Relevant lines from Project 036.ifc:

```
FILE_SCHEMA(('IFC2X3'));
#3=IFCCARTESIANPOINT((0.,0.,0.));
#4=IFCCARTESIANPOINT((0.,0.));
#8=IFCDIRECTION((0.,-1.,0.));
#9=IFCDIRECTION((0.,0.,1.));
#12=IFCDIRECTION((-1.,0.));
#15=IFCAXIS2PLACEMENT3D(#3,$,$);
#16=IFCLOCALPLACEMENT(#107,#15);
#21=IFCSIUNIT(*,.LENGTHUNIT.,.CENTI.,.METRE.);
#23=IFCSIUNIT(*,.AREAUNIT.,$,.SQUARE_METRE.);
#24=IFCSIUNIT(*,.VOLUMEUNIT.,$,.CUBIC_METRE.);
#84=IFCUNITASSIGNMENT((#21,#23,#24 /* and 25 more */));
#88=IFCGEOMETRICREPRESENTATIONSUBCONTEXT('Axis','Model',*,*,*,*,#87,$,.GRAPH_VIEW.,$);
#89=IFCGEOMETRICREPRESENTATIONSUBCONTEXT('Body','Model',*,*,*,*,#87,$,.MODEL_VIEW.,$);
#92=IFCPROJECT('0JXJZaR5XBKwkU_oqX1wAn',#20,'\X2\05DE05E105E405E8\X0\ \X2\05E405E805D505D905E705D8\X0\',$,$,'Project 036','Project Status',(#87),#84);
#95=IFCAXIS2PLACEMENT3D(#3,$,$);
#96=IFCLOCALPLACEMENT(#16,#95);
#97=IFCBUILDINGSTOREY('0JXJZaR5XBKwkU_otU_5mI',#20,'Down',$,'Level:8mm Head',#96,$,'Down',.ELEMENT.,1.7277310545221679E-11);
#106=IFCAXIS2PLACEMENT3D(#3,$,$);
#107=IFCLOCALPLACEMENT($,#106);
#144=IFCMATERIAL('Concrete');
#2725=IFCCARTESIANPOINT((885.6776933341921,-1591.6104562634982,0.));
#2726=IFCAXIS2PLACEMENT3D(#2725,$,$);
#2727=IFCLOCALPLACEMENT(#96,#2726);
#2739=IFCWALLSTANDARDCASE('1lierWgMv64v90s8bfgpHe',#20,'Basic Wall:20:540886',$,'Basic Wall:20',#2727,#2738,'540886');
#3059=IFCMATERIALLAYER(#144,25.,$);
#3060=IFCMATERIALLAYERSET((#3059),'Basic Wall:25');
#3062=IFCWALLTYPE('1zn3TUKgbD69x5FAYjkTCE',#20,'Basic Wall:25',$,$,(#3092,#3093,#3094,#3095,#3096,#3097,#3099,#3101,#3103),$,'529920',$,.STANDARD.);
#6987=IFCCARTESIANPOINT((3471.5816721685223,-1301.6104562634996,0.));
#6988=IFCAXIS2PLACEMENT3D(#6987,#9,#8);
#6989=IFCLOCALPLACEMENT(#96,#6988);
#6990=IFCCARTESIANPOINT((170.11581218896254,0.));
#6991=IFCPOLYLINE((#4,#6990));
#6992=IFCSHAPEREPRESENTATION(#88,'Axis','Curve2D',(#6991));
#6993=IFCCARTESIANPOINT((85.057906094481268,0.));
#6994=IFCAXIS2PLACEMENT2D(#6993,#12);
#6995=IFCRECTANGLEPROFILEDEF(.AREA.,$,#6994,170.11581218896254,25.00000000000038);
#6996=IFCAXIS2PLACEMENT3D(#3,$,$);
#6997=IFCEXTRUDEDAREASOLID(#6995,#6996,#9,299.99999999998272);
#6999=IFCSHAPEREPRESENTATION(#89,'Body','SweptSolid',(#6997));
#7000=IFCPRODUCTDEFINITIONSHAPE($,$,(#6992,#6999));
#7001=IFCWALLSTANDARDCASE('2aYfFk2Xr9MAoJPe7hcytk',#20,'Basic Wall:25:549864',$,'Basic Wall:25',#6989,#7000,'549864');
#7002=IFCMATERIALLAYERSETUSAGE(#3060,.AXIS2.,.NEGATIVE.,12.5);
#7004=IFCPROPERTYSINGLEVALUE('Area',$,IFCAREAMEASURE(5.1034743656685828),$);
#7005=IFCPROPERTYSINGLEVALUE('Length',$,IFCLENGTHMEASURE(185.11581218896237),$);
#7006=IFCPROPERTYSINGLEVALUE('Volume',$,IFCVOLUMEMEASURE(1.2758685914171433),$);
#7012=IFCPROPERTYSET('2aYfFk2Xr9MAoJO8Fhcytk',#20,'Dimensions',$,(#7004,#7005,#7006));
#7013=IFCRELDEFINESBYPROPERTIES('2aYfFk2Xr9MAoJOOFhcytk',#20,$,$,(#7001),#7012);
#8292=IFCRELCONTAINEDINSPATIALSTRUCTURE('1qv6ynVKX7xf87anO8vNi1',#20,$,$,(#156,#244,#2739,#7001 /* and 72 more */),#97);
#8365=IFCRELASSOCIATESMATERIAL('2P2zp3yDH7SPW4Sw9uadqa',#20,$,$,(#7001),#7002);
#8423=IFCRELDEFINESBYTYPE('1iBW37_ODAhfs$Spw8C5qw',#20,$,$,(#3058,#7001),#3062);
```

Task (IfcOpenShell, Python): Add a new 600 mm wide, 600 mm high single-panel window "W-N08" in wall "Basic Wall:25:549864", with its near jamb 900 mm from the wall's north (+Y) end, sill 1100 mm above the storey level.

```python
import numpy as np
import ifcopenshell
import ifcopenshell.api.feature
import ifcopenshell.api.geometry
import ifcopenshell.api.pset
import ifcopenshell.api.root
import ifcopenshell.api.spatial
import ifcopenshell.api.type
import ifcopenshell.geom
import ifcopenshell.util.element
import ifcopenshell.util.placement
import ifcopenshell.util.representation
import ifcopenshell.util.shape
import ifcopenshell.util.unit

model = ifcopenshell.open("Project 036.ifc")
unit_scale = ifcopenshell.util.unit.calculate_unit_scale(model)
area_scale = ifcopenshell.util.unit.calculate_unit_scale(model, "AREAUNIT")
volume_scale = ifcopenshell.util.unit.calculate_unit_scale(model, "VOLUMEUNIT")
settings = ifcopenshell.geom.settings()


def volume(element):
    """Net volume in cubic metres, openings subtracted."""
    shape = ifcopenshell.geom.create_shape(settings, element)
    return ifcopenshell.util.shape.get_volume(shape.geometry)


wall = model.by_guid("2aYfFk2Xr9MAoJPe7hcytk")
storey = ifcopenshell.util.element.get_container(wall, ifc_class="IfcBuildingStorey")
context = ifcopenshell.util.representation.get_context(model, "Model", "Body", "MODEL_VIEW")
before = volume(wall)

width, height, from_end, sill = 0.6, 0.6, 0.9, 1.1  # metres

# The wall runs along its own X axis, and the end named is its -X end.
wall_shape = ifcopenshell.geom.create_shape(settings, wall)
x, y, z = ifcopenshell.util.shape.get_vertices(wall_shape.geometry).T
start = x.min() + from_end
face, thickness = float(y.min()), float(y.max() - y.min())
wall_matrix = ifcopenshell.util.placement.get_local_placement(wall.ObjectPlacement)
level = ifcopenshell.util.placement.get_local_placement(storey.ObjectPlacement)[2, 3]


def in_wall(x, y):
    """Placement at x, y metres in the wall's axes, at sill height."""
    matrix = wall_matrix.copy()
    matrix[:, 3] = wall_matrix @ np.array([x / unit_scale, y / unit_scale, 0.0, 1.0])
    matrix[2, 3] = level + sill / unit_scale
    return matrix


# Opening: a box that overshoots both wall faces by 50 mm.
opening = ifcopenshell.api.root.create_entity(model, ifc_class="IfcOpeningElement")
box = ifcopenshell.api.geometry.add_wall_representation(
    model, context=context, length=width, height=height, thickness=thickness + 0.1
)
ifcopenshell.api.geometry.assign_representation(model, product=opening, representation=box)
ifcopenshell.api.geometry.edit_object_placement(model, product=opening, matrix=in_wall(start, face - 0.05), is_si=False)
ifcopenshell.api.feature.add_feature(model, feature=opening, element=wall)

window = ifcopenshell.api.root.create_entity(model, ifc_class="IfcWindow", name="W-N08")
window.OverallWidth, window.OverallHeight = width / unit_scale, height / unit_scale
body = ifcopenshell.api.geometry.add_window_representation(
    model,
    context=context,
    overall_width=window.OverallWidth,
    overall_height=window.OverallHeight,
    partition_type="SINGLE_PANEL",
)
ifcopenshell.api.geometry.assign_representation(model, product=window, representation=body)
ifcopenshell.api.spatial.assign_container(model, products=[window], relating_structure=storey)
fills = ifcopenshell.api.feature.add_filling(model, opening=opening, element=window)
fills.OwnerHistory = window.OwnerHistory  # required in IFC2X3

# IFC2X3 keeps the operation on the window style.
style = ifcopenshell.api.root.create_entity(model, ifc_class="IfcWindowStyle", name="W-N08")
style.OperationType, style.ConstructionType = "SINGLE_PANEL", "NOTDEFINED"
style.ParameterTakesPrecedence = style.Sizeable = False
ifcopenshell.api.type.assign_type(model, related_objects=[window], relating_type=style)

# Centre the window in the wall's thickness.
ifcopenshell.api.geometry.edit_object_placement(model, product=window, matrix=in_wall(start, face), is_si=False)
window_shape = ifcopenshell.geom.create_shape(settings, window)
depth = ifcopenshell.util.shape.get_vertices(window_shape.geometry)[:, 1]
offset = face + thickness / 2 - (depth.min() + depth.max()) / 2
ifcopenshell.api.geometry.edit_object_placement(model, product=window, matrix=in_wall(start, offset), is_si=False)

after = volume(wall)

# Update the wall's stored quantities.
pset = model.by_id(ifcopenshell.util.element.get_pset(wall, "Dimensions", should_inherit=False)["id"])
ifcopenshell.api.pset.edit_pset(model, pset=pset, properties={
    "Area": model.create_entity("IfcAreaMeasure", after / thickness / area_scale),
    "Volume": model.create_entity("IfcVolumeMeasure", after / volume_scale),
})

print(f"wall volume {before:.3f} -> {after:.3f} m3")

model.write("Project 036_updated.ifc")
```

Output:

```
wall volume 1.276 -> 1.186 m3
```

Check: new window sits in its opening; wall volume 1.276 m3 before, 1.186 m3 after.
